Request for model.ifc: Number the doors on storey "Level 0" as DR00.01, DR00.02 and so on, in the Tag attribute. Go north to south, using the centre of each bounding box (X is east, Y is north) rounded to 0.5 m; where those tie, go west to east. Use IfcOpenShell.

First a look at what the model holds.

```python
import ifcopenshell
import ifcopenshell.util.element
import ifcopenshell.util.placement

model = ifcopenshell.open("model.ifc")
print(model.schema)
storey = next(s for s in model.by_type("IfcBuildingStorey") if s.Name == "Level 0")
doors = [e for e in ifcopenshell.util.element.get_decomposition(storey) if e.is_a("IfcDoor")]
for e in sorted(doors, key=lambda e: e.id()):
    origin = ifcopenshell.util.placement.get_local_placement(e.ObjectPlacement)[:3, 3]
    print(e.id(), e.Tag, e.Name, origin.round(2) + 0.0, sep=" | ")
```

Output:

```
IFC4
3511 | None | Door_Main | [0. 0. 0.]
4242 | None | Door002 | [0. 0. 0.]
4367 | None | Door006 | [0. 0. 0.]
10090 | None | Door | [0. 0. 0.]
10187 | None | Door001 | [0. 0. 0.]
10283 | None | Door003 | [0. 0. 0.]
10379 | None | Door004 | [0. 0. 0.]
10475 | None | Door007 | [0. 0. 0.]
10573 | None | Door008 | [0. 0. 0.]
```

```python
import ifcopenshell
import ifcopenshell.geom
import ifcopenshell.util.element
import ifcopenshell.util.shape

model = ifcopenshell.open("model.ifc")
settings = ifcopenshell.geom.settings()
settings.set("use-world-coords", True)


def centre(element):
    shape = ifcopenshell.geom.create_shape(settings, element)
    return ifcopenshell.util.shape.get_bbox_centroid(shape.geometry)


storey = next(s for s in model.by_type("IfcBuildingStorey") if s.Name == "Level 0")
doors = [e for e in ifcopenshell.util.element.get_decomposition(storey) if e.is_a("IfcDoor")]

# Insertion points can sit at a corner or the storey origin, so sort by the geometry (in metres).
centres = {e: centre(e) for e in doors}
doors.sort(key=lambda e: (-round(centres[e][1] / 0.5), centres[e][0]))

for i, e in enumerate(doors, start=1):
    number = f"DR00.{i:02d}"
    e.Tag = number
    print(e.id(), number)

model.write("model_rev.ifc")
```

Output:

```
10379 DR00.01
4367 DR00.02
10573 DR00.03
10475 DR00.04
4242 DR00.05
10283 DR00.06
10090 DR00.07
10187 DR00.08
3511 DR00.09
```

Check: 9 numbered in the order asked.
